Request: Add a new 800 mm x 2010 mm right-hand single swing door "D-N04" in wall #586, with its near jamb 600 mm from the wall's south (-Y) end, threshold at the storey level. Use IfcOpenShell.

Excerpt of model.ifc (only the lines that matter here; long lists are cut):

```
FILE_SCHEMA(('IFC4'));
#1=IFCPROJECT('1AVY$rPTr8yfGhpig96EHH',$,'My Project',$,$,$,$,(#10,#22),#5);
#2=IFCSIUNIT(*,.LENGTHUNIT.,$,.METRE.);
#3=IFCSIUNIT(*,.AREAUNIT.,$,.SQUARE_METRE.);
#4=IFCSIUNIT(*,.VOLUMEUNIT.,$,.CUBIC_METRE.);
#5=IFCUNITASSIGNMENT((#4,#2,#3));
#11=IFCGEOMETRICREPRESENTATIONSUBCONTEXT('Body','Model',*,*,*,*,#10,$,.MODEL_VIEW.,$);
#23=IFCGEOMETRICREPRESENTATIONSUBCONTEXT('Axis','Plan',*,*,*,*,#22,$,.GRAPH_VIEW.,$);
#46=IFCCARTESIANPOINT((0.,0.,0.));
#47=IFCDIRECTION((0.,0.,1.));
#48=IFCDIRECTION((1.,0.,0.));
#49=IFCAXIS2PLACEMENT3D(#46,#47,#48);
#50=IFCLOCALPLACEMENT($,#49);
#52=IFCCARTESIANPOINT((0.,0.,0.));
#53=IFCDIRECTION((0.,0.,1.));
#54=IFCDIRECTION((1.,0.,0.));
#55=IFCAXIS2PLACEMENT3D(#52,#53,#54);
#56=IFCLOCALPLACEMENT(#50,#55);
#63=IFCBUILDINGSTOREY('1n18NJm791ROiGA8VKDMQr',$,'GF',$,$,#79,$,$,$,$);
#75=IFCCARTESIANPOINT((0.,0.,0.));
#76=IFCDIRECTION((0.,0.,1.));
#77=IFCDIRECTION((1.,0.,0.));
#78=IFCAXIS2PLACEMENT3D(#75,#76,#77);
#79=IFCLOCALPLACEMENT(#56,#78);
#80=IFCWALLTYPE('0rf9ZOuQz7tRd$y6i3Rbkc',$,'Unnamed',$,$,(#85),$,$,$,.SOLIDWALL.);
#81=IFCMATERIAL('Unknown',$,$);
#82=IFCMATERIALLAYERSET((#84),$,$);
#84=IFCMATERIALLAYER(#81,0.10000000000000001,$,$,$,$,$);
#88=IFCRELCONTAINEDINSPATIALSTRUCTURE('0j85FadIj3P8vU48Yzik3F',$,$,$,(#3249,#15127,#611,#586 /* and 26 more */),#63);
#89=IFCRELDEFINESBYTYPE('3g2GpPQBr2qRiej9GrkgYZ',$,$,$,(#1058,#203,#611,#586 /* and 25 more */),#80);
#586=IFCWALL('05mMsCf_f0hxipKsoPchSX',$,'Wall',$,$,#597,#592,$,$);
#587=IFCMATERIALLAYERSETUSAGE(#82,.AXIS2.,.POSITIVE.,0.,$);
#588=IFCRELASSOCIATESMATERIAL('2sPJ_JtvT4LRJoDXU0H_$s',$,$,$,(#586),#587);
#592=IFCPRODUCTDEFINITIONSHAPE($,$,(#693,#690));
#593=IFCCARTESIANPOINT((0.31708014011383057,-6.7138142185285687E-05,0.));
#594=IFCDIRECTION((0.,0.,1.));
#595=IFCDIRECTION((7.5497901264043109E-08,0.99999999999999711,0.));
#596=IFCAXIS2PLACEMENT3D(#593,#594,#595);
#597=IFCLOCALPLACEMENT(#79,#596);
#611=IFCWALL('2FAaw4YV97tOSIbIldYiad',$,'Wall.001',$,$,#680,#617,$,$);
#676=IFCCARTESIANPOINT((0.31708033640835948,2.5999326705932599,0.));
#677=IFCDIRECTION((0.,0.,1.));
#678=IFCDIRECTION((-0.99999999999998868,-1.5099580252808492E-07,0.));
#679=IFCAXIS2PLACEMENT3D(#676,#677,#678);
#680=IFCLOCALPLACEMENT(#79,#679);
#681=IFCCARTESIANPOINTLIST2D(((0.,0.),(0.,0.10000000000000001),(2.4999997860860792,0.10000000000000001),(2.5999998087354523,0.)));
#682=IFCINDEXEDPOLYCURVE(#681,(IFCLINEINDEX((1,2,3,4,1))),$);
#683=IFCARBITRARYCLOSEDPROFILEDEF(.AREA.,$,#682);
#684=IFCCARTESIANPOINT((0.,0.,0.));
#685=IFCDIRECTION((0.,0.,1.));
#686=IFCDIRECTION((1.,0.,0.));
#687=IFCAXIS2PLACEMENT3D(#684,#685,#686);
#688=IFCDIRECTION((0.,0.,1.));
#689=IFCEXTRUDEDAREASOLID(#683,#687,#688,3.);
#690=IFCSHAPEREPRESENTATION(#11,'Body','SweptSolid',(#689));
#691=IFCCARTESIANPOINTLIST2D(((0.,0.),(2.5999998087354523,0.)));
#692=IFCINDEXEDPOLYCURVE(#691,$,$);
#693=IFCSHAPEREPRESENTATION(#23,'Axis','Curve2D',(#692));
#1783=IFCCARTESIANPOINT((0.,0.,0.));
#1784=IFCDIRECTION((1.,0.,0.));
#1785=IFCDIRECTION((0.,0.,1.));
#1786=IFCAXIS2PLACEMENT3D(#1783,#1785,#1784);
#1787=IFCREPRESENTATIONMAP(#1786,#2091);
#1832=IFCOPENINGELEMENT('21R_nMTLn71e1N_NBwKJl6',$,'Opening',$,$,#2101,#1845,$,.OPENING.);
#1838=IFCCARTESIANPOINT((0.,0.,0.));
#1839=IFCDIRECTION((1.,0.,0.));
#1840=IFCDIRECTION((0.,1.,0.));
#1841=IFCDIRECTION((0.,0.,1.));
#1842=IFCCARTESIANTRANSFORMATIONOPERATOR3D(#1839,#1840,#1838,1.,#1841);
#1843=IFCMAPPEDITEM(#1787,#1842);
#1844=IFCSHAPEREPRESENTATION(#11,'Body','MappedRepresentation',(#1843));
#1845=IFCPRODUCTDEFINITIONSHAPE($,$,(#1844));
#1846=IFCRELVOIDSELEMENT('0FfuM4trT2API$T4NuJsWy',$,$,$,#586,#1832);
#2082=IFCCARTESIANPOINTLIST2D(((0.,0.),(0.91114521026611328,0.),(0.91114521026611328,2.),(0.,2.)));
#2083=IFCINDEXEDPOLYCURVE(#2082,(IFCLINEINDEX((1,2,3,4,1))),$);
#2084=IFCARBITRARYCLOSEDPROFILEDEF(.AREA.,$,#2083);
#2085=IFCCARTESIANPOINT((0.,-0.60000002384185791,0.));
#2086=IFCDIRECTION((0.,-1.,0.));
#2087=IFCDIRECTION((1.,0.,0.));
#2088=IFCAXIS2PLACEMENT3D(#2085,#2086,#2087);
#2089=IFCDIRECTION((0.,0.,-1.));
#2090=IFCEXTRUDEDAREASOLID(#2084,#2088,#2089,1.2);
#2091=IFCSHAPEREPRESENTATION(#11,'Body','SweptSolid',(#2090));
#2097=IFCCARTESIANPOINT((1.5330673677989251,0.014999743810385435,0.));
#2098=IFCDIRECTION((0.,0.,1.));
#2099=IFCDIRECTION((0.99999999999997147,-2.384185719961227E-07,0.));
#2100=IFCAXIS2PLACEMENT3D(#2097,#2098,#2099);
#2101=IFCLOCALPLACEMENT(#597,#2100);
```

```python
import numpy as np
import ifcopenshell
import ifcopenshell.api.feature
import ifcopenshell.api.geometry
import ifcopenshell.api.root
import ifcopenshell.api.spatial
import ifcopenshell.geom
import ifcopenshell.util.element
import ifcopenshell.util.placement
import ifcopenshell.util.representation
import ifcopenshell.util.shape
import ifcopenshell.util.unit

model = ifcopenshell.open("model.ifc")
unit_scale = ifcopenshell.util.unit.calculate_unit_scale(model)
settings = ifcopenshell.geom.settings()


def volume(element):
    """Net volume in cubic metres, openings subtracted."""
    shape = ifcopenshell.geom.create_shape(settings, element)
    return ifcopenshell.util.shape.get_volume(shape.geometry)


wall = model.by_guid("05mMsCf_f0hxipKsoPchSX")
storey = ifcopenshell.util.element.get_container(wall, ifc_class="IfcBuildingStorey")
context = ifcopenshell.util.representation.get_context(model, "Model", "Body", "MODEL_VIEW")
before = volume(wall)

width, height, from_end, sill = 0.8, 2.01, 0.6, 0.0  # metres

# The wall runs along its own X axis, and the end named is its -X end.
wall_shape = ifcopenshell.geom.create_shape(settings, wall)
x, y, z = ifcopenshell.util.shape.get_vertices(wall_shape.geometry).T
start = x.min() + from_end
face, thickness = float(y.min()), float(y.max() - y.min())
wall_matrix = ifcopenshell.util.placement.get_local_placement(wall.ObjectPlacement)
level = ifcopenshell.util.placement.get_local_placement(storey.ObjectPlacement)[2, 3]


def in_wall(x, y):
    """Placement at x, y metres in the wall's axes, at sill height."""
    matrix = wall_matrix.copy()
    matrix[:, 3] = wall_matrix @ np.array([x / unit_scale, y / unit_scale, 0.0, 1.0])
    matrix[2, 3] = level + sill / unit_scale
    return matrix


# Opening: a box that overshoots both wall faces by 50 mm.
opening = ifcopenshell.api.root.create_entity(model, ifc_class="IfcOpeningElement", predefined_type="OPENING")
box = ifcopenshell.api.geometry.add_wall_representation(
    model, context=context, length=width, height=height, thickness=thickness + 0.1
)
ifcopenshell.api.geometry.assign_representation(model, product=opening, representation=box)
ifcopenshell.api.geometry.edit_object_placement(model, product=opening, matrix=in_wall(start, face - 0.05), is_si=False)
ifcopenshell.api.feature.add_feature(model, feature=opening, element=wall)

door = ifcopenshell.api.root.create_entity(model, ifc_class="IfcDoor", name="D-N04", predefined_type="DOOR")
door.OverallWidth, door.OverallHeight = width / unit_scale, height / unit_scale
door.OperationType = "SINGLE_SWING_RIGHT"
body = ifcopenshell.api.geometry.add_door_representation(
    model,
    context=context,
    overall_width=door.OverallWidth,
    overall_height=door.OverallHeight,
    operation_type="SINGLE_SWING_RIGHT",
    lining_properties={"LiningDepth": thickness / unit_scale, "ThresholdDepth": thickness / unit_scale},
)
ifcopenshell.api.geometry.assign_representation(model, product=door, representation=body)
ifcopenshell.api.spatial.assign_container(model, products=[door], relating_structure=storey)
ifcopenshell.api.feature.add_filling(model, opening=opening, element=door)

# The lining spans the wall, so the door starts at the wall face.
ifcopenshell.api.geometry.edit_object_placement(model, product=door, matrix=in_wall(start, face), is_si=False)

after = volume(wall)

print(f"wall volume {before:.3f} -> {after:.3f} m3")

model.write("model-out.ifc")
```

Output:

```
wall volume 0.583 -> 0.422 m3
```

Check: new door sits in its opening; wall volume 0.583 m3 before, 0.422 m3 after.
